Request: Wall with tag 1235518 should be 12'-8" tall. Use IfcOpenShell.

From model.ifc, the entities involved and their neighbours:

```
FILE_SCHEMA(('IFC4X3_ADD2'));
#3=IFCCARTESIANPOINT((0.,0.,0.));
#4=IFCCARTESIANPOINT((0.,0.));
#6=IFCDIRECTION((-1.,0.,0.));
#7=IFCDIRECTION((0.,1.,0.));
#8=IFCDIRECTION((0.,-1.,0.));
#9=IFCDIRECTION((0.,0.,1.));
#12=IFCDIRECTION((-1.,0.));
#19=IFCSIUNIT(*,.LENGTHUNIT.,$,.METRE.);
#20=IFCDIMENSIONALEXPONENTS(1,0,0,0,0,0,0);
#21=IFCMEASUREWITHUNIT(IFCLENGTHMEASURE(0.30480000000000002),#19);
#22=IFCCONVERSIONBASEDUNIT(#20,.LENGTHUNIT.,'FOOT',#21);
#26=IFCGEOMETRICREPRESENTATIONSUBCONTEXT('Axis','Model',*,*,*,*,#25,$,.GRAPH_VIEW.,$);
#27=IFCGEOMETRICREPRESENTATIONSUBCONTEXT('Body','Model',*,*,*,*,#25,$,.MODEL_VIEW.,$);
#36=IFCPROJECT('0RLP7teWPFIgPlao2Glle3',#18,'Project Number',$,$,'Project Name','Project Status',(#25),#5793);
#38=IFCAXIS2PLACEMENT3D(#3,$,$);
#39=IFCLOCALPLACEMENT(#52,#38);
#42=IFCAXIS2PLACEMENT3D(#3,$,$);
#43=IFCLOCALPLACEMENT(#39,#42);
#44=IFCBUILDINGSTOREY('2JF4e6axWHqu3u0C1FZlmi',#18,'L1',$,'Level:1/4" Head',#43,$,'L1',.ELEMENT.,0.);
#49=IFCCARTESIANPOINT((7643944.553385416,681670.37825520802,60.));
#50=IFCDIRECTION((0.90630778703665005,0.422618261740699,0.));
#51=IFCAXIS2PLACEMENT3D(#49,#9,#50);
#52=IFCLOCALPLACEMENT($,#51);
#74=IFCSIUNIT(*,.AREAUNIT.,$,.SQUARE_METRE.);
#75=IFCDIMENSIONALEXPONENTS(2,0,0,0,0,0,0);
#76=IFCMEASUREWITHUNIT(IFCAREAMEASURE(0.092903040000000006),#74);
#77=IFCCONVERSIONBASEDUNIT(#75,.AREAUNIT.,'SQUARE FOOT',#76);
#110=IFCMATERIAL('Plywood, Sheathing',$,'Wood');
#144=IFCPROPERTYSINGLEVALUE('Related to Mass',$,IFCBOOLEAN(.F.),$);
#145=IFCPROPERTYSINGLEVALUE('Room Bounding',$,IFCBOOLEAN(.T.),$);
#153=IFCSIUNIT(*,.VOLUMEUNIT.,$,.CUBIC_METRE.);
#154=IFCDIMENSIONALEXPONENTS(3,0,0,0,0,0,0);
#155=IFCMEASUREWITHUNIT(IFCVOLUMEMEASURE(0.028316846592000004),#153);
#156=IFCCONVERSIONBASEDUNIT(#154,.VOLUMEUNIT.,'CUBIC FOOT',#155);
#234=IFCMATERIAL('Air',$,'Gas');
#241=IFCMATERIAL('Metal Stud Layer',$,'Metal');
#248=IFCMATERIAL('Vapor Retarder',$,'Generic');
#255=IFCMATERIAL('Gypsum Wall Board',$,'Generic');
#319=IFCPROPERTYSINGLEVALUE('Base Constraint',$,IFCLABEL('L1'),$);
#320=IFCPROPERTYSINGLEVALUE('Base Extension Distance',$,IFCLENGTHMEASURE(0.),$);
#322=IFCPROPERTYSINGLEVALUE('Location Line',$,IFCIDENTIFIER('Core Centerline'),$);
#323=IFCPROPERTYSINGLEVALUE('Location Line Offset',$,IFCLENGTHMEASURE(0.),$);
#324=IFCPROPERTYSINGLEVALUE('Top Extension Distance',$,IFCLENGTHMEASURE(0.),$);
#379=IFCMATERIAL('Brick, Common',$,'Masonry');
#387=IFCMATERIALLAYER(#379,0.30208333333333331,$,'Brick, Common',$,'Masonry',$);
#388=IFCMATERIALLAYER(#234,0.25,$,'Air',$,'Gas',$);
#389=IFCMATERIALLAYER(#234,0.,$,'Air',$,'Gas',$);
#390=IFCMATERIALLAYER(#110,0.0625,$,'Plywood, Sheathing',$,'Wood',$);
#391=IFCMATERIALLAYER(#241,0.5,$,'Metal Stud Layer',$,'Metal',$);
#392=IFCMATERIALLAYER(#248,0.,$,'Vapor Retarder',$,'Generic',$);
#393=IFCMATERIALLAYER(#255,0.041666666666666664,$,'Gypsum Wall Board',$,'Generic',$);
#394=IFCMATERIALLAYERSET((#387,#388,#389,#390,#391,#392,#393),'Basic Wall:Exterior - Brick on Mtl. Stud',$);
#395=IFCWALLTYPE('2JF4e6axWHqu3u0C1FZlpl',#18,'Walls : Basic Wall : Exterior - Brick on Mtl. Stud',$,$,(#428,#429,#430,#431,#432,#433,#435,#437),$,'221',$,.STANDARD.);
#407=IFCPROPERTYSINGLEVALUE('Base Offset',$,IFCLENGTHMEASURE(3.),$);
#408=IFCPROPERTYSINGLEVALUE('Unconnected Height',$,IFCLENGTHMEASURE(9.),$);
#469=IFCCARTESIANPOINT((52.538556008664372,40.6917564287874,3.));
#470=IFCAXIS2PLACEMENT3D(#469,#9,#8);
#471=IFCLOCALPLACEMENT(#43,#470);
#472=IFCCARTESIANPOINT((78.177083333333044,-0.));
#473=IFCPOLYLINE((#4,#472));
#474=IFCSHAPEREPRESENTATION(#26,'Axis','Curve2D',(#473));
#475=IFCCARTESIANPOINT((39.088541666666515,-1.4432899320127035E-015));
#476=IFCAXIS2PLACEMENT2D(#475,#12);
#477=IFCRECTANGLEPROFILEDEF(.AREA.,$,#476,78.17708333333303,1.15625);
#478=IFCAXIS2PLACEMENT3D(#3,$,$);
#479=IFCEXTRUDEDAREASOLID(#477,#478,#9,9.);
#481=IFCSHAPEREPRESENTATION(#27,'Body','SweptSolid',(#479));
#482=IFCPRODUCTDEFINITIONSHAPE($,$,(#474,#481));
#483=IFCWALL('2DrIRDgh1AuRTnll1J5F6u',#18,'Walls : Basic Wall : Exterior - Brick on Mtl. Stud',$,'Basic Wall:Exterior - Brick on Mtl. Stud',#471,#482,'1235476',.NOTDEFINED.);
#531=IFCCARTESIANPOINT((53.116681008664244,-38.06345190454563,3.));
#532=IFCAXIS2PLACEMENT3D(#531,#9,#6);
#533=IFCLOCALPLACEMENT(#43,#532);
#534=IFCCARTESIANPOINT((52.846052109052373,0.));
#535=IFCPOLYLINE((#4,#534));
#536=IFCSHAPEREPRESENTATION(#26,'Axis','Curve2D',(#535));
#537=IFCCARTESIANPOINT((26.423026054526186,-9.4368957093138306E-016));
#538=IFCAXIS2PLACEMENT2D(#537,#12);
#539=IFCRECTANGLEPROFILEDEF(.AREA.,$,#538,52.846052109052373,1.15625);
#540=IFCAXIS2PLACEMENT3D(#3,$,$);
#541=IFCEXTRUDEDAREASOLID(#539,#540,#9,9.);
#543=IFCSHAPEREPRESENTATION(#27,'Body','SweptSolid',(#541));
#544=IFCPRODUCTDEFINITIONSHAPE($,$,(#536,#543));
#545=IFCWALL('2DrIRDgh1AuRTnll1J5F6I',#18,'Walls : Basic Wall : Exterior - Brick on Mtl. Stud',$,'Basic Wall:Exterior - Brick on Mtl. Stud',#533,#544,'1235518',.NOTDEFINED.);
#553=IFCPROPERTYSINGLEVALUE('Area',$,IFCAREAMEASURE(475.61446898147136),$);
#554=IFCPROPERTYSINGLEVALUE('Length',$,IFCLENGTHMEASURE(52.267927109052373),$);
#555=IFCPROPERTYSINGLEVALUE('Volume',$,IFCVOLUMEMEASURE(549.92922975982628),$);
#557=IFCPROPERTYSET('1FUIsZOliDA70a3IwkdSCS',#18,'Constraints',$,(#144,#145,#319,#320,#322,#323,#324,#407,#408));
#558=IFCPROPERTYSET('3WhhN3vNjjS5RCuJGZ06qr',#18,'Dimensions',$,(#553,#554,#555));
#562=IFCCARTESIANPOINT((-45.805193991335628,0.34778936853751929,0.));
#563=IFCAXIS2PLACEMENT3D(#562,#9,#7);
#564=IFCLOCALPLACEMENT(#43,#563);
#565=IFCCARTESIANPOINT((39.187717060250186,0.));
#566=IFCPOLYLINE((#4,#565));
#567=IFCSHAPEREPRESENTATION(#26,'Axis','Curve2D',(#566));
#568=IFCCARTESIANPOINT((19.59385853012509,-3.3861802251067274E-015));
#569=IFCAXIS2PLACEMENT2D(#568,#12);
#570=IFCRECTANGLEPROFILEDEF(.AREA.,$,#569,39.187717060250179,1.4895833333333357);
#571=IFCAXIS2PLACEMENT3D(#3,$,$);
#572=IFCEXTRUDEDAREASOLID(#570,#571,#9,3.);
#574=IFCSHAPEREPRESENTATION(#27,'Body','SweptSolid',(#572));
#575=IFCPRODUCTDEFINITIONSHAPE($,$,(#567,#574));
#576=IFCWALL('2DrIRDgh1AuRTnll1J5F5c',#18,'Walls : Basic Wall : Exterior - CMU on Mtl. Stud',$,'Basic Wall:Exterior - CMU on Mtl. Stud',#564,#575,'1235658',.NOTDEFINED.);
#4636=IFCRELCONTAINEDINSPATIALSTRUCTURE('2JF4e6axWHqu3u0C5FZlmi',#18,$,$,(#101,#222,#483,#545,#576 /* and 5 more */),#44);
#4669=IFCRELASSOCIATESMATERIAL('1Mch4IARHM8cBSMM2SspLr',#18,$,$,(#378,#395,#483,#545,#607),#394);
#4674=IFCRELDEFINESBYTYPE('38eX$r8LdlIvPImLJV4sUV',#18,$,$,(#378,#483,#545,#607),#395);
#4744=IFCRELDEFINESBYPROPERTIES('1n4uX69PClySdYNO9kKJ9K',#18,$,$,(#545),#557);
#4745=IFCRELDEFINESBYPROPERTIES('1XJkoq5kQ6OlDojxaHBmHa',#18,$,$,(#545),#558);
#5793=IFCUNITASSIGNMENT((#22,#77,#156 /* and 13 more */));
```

```python
import ifcopenshell
import ifcopenshell.api.pset
import ifcopenshell.geom
import ifcopenshell.util.element
import ifcopenshell.util.representation
import ifcopenshell.util.shape
import ifcopenshell.util.unit

model = ifcopenshell.open("model.ifc")
unit_scale = ifcopenshell.util.unit.calculate_unit_scale(model)
area_scale = ifcopenshell.util.unit.calculate_unit_scale(model, "AREAUNIT")
volume_scale = ifcopenshell.util.unit.calculate_unit_scale(model, "VOLUMEUNIT")
settings = ifcopenshell.geom.settings()


def volume(element):
    """Net volume in cubic metres, openings subtracted."""
    shape = ifcopenshell.geom.create_shape(settings, element)
    return ifcopenshell.util.shape.get_volume(shape.geometry)


wall = model.by_guid("2DrIRDgh1AuRTnll1J5F6I")
before = volume(wall)

body = ifcopenshell.util.representation.get_representation(wall, "Model", "Body")
solid = body.Items[0]
old_height = solid.Depth
solid.Depth = 152 * 0.0254 / unit_scale
after = volume(wall)
thickness = 0.3524  # wall thickness in metres

# Update the stored height, areas and volumes.
pset = model.by_id(ifcopenshell.util.element.get_pset(wall, "Constraints", should_inherit=False)["id"])
ifcopenshell.api.pset.edit_pset(model, pset=pset, properties={
    "Unconnected Height": model.create_entity("IfcLengthMeasure", solid.Depth),
})
pset = model.by_id(ifcopenshell.util.element.get_pset(wall, "Dimensions", should_inherit=False)["id"])
ifcopenshell.api.pset.edit_pset(model, pset=pset, properties={
    "Area": model.create_entity("IfcAreaMeasure", after / thickness / area_scale),
    "Volume": model.create_entity("IfcVolumeMeasure", after / volume_scale),
})

print(f"height {old_height:g} -> {solid.Depth:g}, volume {before:.3f} -> {after:.3f} m3")

model.write("model_rev.ifc")
```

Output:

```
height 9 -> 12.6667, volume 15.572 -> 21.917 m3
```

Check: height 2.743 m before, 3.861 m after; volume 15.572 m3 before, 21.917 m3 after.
